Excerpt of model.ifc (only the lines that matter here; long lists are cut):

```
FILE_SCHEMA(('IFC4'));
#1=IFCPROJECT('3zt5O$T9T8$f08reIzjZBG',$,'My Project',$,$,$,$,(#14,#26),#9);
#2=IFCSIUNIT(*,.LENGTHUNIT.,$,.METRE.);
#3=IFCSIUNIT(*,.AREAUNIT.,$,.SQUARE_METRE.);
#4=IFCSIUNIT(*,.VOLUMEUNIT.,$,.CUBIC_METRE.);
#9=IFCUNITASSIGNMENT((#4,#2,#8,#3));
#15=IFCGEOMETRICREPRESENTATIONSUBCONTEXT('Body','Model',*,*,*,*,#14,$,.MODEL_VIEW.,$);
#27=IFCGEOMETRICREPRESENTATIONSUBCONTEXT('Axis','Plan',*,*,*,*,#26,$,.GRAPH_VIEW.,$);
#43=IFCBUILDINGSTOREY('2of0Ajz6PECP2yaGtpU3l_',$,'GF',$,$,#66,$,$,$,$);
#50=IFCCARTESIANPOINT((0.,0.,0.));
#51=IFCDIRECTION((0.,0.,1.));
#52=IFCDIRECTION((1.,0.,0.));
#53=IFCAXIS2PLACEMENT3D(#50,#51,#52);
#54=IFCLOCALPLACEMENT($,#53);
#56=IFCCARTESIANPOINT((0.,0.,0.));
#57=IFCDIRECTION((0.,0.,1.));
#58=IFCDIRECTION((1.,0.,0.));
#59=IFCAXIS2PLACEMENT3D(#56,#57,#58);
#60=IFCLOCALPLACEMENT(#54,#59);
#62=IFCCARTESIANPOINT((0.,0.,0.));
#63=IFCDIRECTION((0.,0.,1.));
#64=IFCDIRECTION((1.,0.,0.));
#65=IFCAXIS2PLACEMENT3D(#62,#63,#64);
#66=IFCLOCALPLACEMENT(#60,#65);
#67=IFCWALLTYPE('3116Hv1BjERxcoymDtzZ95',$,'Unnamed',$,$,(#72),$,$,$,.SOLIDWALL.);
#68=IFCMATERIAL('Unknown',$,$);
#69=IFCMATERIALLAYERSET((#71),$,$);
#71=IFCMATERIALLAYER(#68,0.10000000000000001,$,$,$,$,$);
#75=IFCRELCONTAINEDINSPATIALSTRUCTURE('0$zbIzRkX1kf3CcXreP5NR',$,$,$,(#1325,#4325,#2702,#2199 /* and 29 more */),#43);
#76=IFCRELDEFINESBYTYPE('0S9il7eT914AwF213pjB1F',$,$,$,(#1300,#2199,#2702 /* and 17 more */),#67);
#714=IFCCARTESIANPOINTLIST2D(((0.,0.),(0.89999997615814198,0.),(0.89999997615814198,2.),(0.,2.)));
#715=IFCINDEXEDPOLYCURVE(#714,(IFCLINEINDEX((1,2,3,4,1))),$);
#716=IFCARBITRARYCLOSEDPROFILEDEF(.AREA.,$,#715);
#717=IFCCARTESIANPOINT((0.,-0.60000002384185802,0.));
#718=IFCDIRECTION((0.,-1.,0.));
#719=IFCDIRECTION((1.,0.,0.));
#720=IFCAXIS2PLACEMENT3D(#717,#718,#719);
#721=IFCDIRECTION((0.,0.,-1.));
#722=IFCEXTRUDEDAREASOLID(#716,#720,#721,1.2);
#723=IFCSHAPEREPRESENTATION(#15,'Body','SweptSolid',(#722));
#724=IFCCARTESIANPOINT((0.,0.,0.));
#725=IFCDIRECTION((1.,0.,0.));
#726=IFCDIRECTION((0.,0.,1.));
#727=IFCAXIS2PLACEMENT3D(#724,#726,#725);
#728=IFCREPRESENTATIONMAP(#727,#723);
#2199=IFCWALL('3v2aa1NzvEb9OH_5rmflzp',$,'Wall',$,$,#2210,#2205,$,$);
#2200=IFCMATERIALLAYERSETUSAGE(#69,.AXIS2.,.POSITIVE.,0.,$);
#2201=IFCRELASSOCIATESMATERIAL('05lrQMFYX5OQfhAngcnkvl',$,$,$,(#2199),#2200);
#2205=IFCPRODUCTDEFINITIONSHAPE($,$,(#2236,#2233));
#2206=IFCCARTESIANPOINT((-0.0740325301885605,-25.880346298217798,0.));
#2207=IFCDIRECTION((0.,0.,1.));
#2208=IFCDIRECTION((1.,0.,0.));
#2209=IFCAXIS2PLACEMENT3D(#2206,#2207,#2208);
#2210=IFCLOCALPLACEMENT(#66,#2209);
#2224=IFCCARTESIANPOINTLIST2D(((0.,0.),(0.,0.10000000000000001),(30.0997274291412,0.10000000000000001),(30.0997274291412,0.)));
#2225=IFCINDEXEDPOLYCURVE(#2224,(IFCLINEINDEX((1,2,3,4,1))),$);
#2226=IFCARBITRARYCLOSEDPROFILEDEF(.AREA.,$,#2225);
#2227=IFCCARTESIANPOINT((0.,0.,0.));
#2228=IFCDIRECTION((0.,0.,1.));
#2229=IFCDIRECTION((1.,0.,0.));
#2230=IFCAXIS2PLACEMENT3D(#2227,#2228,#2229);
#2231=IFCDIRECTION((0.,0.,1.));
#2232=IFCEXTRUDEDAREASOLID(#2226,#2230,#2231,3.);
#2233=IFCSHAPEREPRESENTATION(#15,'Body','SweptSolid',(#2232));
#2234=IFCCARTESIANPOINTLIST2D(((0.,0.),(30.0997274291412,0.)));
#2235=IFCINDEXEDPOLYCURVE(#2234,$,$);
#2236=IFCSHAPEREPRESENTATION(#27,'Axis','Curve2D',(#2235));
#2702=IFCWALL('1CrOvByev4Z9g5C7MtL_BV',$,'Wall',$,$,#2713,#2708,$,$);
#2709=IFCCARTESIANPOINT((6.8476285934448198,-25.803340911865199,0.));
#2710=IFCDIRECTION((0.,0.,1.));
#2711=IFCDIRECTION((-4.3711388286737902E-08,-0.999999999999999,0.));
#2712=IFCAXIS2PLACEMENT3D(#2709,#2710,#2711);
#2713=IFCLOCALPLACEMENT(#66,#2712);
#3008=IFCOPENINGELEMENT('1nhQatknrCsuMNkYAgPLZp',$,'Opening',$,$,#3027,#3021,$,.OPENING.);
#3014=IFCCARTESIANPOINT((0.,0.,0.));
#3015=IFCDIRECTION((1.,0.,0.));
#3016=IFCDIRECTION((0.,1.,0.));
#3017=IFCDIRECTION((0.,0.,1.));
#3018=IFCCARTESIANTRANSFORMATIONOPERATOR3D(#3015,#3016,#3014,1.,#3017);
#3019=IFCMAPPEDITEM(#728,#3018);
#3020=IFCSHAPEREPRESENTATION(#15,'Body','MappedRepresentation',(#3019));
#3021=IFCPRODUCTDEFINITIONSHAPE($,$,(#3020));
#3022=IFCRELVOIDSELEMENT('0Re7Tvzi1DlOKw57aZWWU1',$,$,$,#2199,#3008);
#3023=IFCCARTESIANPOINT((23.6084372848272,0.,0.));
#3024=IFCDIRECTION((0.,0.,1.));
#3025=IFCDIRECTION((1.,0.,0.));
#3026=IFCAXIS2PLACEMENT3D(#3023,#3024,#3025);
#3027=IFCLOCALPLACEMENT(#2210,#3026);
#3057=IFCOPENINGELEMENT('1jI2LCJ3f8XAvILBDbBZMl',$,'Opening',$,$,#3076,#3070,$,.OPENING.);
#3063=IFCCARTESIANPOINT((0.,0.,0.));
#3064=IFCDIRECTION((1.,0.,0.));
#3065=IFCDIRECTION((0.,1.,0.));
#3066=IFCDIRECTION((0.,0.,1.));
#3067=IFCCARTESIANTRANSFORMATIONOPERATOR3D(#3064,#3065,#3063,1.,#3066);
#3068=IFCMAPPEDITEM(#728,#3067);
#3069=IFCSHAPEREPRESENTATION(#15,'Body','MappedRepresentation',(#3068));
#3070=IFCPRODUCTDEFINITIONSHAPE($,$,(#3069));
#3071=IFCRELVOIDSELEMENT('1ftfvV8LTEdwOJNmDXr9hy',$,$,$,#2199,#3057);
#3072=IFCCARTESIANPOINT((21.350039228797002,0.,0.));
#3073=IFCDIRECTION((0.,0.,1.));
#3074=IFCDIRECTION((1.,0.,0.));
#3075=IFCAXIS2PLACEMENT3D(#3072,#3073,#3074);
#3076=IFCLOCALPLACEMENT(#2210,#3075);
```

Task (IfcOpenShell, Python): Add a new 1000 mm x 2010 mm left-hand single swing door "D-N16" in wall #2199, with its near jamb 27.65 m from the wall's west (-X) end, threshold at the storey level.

```python
import numpy as np
import ifcopenshell
import ifcopenshell.api.feature
import ifcopenshell.api.geometry
import ifcopenshell.api.root
import ifcopenshell.api.spatial
import ifcopenshell.geom
import ifcopenshell.util.element
import ifcopenshell.util.placement
import ifcopenshell.util.representation
import ifcopenshell.util.shape
import ifcopenshell.util.unit

model = ifcopenshell.open("model.ifc")
unit_scale = ifcopenshell.util.unit.calculate_unit_scale(model)
settings = ifcopenshell.geom.settings()


def volume(element):
    """Net volume in cubic metres, openings subtracted."""
    shape = ifcopenshell.geom.create_shape(settings, element)
    return ifcopenshell.util.shape.get_volume(shape.geometry)


wall = model.by_guid("3v2aa1NzvEb9OH_5rmflzp")
storey = ifcopenshell.util.element.get_container(wall, ifc_class="IfcBuildingStorey")
context = ifcopenshell.util.representation.get_context(model, "Model", "Body", "MODEL_VIEW")
before = volume(wall)

width, height, from_end, sill = 1, 2.01, 27.65, 0.0  # metres

# The wall runs along its own X axis, and the end named is its -X end.
wall_shape = ifcopenshell.geom.create_shape(settings, wall)
x, y, z = ifcopenshell.util.shape.get_vertices(wall_shape.geometry).T
start = x.min() + from_end
face, thickness = float(y.min()), float(y.max() - y.min())
wall_matrix = ifcopenshell.util.placement.get_local_placement(wall.ObjectPlacement)
level = ifcopenshell.util.placement.get_local_placement(storey.ObjectPlacement)[2, 3]


def in_wall(x, y):
    """Placement at x, y metres in the wall's axes, at sill height."""
    matrix = wall_matrix.copy()
    matrix[:, 3] = wall_matrix @ np.array([x / unit_scale, y / unit_scale, 0.0, 1.0])
    matrix[2, 3] = level + sill / unit_scale
    return matrix


# Opening: a box that overshoots both wall faces by 50 mm.
opening = ifcopenshell.api.root.create_entity(model, ifc_class="IfcOpeningElement", predefined_type="OPENING")
box = ifcopenshell.api.geometry.add_wall_representation(
    model, context=context, length=width, height=height, thickness=thickness + 0.1
)
ifcopenshell.api.geometry.assign_representation(model, product=opening, representation=box)
ifcopenshell.api.geometry.edit_object_placement(model, product=opening, matrix=in_wall(start, face - 0.05), is_si=False)
ifcopenshell.api.feature.add_feature(model, feature=opening, element=wall)

door = ifcopenshell.api.root.create_entity(model, ifc_class="IfcDoor", name="D-N16", predefined_type="DOOR")
door.OverallWidth, door.OverallHeight = width / unit_scale, height / unit_scale
door.OperationType = "SINGLE_SWING_LEFT"
body = ifcopenshell.api.geometry.add_door_representation(
    model,
    context=context,
    overall_width=door.OverallWidth,
    overall_height=door.OverallHeight,
    operation_type="SINGLE_SWING_LEFT",
    lining_properties={"LiningDepth": thickness / unit_scale, "ThresholdDepth": thickness / unit_scale},
)
ifcopenshell.api.geometry.assign_representation(model, product=door, representation=body)
ifcopenshell.api.spatial.assign_container(model, products=[door], relating_structure=storey)
ifcopenshell.api.feature.add_filling(model, opening=opening, element=door)

# The lining spans the wall, so the door starts at the wall face.
ifcopenshell.api.geometry.edit_object_placement(model, product=door, matrix=in_wall(start, face), is_si=False)

after = volume(wall)

print(f"wall volume {before:.3f} -> {after:.3f} m3")

model.write("model_v2.ifc")
```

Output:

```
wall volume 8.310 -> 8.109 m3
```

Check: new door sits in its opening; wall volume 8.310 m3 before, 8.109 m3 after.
